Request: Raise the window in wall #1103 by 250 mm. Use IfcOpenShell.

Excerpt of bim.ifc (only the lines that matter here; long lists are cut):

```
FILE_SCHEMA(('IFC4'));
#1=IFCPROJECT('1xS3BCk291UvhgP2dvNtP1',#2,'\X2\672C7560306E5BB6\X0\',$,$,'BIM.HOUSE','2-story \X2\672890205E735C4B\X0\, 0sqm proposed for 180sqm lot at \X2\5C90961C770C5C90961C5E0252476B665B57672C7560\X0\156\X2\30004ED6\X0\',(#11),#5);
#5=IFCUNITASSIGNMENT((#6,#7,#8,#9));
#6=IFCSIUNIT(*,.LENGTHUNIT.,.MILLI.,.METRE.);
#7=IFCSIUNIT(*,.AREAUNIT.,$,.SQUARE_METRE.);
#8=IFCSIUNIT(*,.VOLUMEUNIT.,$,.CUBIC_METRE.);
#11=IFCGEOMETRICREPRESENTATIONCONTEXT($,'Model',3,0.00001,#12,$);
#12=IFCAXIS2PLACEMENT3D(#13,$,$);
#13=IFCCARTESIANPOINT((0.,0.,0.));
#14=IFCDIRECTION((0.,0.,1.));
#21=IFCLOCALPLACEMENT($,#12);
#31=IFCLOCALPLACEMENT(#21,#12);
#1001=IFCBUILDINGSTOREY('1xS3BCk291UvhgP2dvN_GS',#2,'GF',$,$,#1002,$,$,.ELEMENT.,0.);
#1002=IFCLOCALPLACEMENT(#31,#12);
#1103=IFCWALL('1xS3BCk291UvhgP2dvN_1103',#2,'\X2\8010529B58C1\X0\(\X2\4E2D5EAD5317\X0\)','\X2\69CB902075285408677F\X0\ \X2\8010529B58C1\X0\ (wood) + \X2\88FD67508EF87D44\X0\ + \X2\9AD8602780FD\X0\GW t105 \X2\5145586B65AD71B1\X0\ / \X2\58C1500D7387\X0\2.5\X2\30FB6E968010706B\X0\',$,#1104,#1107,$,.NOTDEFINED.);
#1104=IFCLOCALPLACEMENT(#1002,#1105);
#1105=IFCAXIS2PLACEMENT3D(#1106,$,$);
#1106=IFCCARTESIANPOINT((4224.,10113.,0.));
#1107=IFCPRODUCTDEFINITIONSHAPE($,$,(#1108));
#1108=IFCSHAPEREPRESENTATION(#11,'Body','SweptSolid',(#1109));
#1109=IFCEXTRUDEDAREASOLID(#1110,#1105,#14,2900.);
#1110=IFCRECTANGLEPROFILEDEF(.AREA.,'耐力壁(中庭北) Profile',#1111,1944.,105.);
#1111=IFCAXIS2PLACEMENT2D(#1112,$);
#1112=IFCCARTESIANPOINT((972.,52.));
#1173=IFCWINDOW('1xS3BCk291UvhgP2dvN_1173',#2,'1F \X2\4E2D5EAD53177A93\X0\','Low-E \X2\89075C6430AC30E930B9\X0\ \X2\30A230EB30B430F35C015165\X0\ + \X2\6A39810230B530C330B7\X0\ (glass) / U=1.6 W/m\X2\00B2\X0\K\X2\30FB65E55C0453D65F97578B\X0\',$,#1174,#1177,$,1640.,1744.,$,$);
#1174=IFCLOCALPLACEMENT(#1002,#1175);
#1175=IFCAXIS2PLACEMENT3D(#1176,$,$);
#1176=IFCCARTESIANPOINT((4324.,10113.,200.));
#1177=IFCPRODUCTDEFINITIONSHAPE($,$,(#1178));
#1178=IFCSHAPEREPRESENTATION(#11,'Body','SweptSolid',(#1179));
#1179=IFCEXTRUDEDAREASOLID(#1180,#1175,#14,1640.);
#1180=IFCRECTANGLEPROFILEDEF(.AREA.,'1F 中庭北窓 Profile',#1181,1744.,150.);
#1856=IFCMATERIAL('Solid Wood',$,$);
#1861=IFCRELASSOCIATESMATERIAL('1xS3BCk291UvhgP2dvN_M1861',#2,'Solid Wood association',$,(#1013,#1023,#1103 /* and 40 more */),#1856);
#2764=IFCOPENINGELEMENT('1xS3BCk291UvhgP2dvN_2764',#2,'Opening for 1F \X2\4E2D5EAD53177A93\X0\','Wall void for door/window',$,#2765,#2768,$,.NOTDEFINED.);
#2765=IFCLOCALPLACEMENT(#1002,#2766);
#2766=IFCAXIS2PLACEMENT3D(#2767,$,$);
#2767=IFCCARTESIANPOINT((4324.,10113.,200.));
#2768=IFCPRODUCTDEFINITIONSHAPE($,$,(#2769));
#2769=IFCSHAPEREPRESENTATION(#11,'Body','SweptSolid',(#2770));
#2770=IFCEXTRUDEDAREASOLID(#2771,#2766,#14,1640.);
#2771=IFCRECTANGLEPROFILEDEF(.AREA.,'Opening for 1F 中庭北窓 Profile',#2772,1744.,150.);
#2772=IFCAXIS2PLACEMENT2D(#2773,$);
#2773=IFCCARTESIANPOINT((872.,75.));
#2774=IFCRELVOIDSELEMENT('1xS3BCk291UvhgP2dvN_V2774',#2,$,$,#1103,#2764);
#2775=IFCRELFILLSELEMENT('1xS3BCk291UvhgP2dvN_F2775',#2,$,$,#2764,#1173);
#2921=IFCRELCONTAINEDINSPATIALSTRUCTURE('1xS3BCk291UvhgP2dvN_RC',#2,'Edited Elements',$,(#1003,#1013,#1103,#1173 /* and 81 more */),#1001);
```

```python
import numpy as np
import ifcopenshell
import ifcopenshell.api.geometry
import ifcopenshell.util.placement
import ifcopenshell.util.unit

model = ifcopenshell.open("bim.ifc")
unit_scale = ifcopenshell.util.unit.calculate_unit_scale(model)

window = model.by_id(1173)
opening = window.FillsVoids[0].RelatingOpeningElement
dz = 0.25 / unit_scale

shift = np.array([0.0, 0.0, dz])
# The window is not placed relative to its opening, so move both.
for product in (opening, window):
    matrix = ifcopenshell.util.placement.get_local_placement(product.ObjectPlacement)
    matrix[:3, 3] += shift
    ifcopenshell.api.geometry.edit_object_placement(model, product=product, matrix=matrix, is_si=False)

print(f"moved by {dz * unit_scale:+.3f} m")

model.write("bim_edited.ifc")
```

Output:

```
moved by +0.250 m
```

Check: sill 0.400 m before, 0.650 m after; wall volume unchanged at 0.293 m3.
